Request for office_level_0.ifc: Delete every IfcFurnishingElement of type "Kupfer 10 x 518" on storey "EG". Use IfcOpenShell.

First a look at what the model holds.

```python
import ifcopenshell
import ifcopenshell.util.element

model = ifcopenshell.open("office_level_0.ifc")
print(model.schema)
storey = next(s for s in model.by_type("IfcBuildingStorey") if s.Name == "EG")
furniture = [e for e in ifcopenshell.util.element.get_decomposition(storey) if e.is_a("IfcFurnishingElement")]
seen = {}
for e in furniture:
    element_type = ifcopenshell.util.element.get_type(e)
    name = element_type.Name if element_type not in (None, e) else None
    seen[name] = seen.get(name, 0) + 1
for name, count in sorted(seen.items(), key=str):
    print(count, "x", name)
```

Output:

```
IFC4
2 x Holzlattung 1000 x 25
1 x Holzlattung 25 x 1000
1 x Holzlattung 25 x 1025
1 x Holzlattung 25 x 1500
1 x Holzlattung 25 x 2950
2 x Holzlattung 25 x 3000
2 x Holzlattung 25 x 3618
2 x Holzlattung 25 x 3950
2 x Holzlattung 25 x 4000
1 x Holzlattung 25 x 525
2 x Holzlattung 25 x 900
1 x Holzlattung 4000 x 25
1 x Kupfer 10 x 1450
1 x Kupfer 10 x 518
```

```python
import ifcopenshell
import ifcopenshell.api.root
import ifcopenshell.util.element

model = ifcopenshell.open("office_level_0.ifc")

storey = next(s for s in model.by_type("IfcBuildingStorey") if s.Name == "EG")
furniture = [e for e in ifcopenshell.util.element.get_decomposition(storey) if e.is_a("IfcFurnishingElement")]
targets = [e for e in furniture if (t := ifcopenshell.util.element.get_type(e)) not in (None, e) and t.Name == "Kupfer 10 x 518"]

for e in targets:
    ifcopenshell.api.root.remove_product(model, product=e)
print(len(targets), "removed")

model.write("office_level_0_edited.ifc")
```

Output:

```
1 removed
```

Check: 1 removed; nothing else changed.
